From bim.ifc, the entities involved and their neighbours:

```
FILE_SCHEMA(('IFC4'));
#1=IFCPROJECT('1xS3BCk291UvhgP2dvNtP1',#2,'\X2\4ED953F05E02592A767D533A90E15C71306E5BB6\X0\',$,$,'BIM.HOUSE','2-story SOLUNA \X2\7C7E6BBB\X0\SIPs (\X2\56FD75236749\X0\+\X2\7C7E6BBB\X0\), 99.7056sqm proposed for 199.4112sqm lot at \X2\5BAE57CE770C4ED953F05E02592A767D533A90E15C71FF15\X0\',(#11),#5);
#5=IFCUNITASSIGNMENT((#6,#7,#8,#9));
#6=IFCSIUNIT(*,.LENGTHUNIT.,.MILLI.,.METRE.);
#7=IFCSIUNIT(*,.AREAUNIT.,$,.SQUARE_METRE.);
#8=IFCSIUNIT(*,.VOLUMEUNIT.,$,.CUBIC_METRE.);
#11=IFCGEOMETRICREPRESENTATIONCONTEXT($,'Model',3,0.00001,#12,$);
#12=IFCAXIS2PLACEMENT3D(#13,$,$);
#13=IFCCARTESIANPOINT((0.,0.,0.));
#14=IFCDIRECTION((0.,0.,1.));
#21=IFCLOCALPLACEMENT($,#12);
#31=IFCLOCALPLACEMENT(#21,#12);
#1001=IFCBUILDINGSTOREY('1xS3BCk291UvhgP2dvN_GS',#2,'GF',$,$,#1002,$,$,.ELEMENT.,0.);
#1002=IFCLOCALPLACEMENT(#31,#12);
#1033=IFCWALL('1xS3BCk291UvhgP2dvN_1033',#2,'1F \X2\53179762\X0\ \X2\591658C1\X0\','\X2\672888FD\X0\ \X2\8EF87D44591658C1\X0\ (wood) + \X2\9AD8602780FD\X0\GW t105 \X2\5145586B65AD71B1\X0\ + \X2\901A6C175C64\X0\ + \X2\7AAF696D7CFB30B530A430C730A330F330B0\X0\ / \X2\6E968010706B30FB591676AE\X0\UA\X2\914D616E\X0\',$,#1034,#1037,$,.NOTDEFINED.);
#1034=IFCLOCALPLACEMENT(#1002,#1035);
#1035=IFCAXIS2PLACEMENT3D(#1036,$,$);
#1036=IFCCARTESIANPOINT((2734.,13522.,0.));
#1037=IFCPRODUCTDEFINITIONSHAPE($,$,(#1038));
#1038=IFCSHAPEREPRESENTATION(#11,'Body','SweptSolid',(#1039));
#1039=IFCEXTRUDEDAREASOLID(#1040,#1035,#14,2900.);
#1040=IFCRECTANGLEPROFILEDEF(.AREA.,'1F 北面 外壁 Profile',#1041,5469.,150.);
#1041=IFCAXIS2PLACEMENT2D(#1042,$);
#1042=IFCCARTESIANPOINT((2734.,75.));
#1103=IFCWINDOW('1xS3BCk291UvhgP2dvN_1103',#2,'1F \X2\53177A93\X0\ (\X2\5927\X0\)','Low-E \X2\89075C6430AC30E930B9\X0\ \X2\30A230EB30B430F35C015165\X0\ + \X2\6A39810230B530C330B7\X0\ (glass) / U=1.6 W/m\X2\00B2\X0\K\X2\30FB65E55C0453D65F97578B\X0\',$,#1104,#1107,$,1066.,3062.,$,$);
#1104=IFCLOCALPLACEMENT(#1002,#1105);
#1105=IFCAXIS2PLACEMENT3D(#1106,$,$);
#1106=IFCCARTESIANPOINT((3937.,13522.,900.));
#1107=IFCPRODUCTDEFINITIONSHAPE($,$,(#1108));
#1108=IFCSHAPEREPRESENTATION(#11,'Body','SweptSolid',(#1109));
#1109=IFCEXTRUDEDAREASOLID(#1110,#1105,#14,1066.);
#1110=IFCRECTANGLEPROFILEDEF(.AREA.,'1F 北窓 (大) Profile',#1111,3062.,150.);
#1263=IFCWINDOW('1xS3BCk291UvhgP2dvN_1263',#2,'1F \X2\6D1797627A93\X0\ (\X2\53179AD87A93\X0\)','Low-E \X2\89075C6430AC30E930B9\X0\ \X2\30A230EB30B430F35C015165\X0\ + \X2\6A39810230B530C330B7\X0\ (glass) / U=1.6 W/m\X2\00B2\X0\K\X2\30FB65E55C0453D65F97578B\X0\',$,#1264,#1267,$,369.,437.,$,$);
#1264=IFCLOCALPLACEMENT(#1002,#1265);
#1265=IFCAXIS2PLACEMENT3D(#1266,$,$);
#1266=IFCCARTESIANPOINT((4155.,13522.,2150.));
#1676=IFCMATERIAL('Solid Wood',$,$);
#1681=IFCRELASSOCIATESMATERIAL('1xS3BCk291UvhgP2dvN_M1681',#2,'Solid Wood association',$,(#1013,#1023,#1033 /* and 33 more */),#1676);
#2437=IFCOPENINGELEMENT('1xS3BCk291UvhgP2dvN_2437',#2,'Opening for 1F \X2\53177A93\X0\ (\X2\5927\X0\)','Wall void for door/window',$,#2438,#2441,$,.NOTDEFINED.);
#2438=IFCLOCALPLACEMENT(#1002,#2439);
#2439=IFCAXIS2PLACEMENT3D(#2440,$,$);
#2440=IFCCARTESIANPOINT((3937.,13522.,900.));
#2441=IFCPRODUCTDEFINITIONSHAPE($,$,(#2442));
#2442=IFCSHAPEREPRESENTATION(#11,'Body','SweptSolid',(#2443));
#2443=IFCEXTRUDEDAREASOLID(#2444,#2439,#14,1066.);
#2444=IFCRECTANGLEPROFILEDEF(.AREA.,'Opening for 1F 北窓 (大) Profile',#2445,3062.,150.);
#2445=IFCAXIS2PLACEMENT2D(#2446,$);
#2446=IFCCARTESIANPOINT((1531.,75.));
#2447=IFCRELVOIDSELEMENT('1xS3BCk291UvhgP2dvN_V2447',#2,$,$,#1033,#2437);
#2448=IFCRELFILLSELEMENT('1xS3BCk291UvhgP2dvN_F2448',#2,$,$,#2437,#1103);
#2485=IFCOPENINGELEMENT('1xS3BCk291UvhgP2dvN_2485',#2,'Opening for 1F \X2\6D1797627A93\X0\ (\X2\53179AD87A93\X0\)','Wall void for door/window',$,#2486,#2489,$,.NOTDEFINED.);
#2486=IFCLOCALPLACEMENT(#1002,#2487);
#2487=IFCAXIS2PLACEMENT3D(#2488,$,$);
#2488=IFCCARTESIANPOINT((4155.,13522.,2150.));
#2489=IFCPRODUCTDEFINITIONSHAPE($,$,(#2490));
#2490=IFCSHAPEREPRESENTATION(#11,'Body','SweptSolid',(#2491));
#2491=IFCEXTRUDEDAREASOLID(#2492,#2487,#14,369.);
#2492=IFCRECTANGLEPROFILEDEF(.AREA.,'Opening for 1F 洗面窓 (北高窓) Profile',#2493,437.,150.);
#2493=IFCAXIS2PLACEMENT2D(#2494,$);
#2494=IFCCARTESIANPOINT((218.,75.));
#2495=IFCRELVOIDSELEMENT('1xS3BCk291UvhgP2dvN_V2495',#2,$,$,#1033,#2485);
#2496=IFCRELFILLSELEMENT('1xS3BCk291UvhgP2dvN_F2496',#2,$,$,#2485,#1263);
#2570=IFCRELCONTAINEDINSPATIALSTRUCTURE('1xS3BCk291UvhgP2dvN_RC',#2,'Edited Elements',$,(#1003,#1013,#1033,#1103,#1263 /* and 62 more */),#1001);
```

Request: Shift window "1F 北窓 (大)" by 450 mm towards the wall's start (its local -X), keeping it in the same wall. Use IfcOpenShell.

```python
import ifcopenshell
import ifcopenshell.api.geometry
import ifcopenshell.util.placement

model = ifcopenshell.open("bim.ifc")

window = model.by_id(1103)
opening = window.FillsVoids[0].RelatingOpeningElement
wall = opening.VoidsElements[0].RelatingBuildingElement

wall_matrix = ifcopenshell.util.placement.get_local_placement(wall.ObjectPlacement)
shift = wall_matrix[:3, 0] * -450.0
before = ifcopenshell.util.placement.get_local_placement(window.ObjectPlacement)[:3, 3].copy()

# The window is not placed relative to its opening, so move both.
for product in (opening, window):
    matrix = ifcopenshell.util.placement.get_local_placement(product.ObjectPlacement)
    matrix[:3, 3] += shift
    ifcopenshell.api.geometry.edit_object_placement(model, product=product, matrix=matrix, is_si=False)

after = ifcopenshell.util.placement.get_local_placement(window.ObjectPlacement)[:3, 3]
print("window moved by", (after - before).round(3) + 0.0)

model.write("bim_v2.ifc")
```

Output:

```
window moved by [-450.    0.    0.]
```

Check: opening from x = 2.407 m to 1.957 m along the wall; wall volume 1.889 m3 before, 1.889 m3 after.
